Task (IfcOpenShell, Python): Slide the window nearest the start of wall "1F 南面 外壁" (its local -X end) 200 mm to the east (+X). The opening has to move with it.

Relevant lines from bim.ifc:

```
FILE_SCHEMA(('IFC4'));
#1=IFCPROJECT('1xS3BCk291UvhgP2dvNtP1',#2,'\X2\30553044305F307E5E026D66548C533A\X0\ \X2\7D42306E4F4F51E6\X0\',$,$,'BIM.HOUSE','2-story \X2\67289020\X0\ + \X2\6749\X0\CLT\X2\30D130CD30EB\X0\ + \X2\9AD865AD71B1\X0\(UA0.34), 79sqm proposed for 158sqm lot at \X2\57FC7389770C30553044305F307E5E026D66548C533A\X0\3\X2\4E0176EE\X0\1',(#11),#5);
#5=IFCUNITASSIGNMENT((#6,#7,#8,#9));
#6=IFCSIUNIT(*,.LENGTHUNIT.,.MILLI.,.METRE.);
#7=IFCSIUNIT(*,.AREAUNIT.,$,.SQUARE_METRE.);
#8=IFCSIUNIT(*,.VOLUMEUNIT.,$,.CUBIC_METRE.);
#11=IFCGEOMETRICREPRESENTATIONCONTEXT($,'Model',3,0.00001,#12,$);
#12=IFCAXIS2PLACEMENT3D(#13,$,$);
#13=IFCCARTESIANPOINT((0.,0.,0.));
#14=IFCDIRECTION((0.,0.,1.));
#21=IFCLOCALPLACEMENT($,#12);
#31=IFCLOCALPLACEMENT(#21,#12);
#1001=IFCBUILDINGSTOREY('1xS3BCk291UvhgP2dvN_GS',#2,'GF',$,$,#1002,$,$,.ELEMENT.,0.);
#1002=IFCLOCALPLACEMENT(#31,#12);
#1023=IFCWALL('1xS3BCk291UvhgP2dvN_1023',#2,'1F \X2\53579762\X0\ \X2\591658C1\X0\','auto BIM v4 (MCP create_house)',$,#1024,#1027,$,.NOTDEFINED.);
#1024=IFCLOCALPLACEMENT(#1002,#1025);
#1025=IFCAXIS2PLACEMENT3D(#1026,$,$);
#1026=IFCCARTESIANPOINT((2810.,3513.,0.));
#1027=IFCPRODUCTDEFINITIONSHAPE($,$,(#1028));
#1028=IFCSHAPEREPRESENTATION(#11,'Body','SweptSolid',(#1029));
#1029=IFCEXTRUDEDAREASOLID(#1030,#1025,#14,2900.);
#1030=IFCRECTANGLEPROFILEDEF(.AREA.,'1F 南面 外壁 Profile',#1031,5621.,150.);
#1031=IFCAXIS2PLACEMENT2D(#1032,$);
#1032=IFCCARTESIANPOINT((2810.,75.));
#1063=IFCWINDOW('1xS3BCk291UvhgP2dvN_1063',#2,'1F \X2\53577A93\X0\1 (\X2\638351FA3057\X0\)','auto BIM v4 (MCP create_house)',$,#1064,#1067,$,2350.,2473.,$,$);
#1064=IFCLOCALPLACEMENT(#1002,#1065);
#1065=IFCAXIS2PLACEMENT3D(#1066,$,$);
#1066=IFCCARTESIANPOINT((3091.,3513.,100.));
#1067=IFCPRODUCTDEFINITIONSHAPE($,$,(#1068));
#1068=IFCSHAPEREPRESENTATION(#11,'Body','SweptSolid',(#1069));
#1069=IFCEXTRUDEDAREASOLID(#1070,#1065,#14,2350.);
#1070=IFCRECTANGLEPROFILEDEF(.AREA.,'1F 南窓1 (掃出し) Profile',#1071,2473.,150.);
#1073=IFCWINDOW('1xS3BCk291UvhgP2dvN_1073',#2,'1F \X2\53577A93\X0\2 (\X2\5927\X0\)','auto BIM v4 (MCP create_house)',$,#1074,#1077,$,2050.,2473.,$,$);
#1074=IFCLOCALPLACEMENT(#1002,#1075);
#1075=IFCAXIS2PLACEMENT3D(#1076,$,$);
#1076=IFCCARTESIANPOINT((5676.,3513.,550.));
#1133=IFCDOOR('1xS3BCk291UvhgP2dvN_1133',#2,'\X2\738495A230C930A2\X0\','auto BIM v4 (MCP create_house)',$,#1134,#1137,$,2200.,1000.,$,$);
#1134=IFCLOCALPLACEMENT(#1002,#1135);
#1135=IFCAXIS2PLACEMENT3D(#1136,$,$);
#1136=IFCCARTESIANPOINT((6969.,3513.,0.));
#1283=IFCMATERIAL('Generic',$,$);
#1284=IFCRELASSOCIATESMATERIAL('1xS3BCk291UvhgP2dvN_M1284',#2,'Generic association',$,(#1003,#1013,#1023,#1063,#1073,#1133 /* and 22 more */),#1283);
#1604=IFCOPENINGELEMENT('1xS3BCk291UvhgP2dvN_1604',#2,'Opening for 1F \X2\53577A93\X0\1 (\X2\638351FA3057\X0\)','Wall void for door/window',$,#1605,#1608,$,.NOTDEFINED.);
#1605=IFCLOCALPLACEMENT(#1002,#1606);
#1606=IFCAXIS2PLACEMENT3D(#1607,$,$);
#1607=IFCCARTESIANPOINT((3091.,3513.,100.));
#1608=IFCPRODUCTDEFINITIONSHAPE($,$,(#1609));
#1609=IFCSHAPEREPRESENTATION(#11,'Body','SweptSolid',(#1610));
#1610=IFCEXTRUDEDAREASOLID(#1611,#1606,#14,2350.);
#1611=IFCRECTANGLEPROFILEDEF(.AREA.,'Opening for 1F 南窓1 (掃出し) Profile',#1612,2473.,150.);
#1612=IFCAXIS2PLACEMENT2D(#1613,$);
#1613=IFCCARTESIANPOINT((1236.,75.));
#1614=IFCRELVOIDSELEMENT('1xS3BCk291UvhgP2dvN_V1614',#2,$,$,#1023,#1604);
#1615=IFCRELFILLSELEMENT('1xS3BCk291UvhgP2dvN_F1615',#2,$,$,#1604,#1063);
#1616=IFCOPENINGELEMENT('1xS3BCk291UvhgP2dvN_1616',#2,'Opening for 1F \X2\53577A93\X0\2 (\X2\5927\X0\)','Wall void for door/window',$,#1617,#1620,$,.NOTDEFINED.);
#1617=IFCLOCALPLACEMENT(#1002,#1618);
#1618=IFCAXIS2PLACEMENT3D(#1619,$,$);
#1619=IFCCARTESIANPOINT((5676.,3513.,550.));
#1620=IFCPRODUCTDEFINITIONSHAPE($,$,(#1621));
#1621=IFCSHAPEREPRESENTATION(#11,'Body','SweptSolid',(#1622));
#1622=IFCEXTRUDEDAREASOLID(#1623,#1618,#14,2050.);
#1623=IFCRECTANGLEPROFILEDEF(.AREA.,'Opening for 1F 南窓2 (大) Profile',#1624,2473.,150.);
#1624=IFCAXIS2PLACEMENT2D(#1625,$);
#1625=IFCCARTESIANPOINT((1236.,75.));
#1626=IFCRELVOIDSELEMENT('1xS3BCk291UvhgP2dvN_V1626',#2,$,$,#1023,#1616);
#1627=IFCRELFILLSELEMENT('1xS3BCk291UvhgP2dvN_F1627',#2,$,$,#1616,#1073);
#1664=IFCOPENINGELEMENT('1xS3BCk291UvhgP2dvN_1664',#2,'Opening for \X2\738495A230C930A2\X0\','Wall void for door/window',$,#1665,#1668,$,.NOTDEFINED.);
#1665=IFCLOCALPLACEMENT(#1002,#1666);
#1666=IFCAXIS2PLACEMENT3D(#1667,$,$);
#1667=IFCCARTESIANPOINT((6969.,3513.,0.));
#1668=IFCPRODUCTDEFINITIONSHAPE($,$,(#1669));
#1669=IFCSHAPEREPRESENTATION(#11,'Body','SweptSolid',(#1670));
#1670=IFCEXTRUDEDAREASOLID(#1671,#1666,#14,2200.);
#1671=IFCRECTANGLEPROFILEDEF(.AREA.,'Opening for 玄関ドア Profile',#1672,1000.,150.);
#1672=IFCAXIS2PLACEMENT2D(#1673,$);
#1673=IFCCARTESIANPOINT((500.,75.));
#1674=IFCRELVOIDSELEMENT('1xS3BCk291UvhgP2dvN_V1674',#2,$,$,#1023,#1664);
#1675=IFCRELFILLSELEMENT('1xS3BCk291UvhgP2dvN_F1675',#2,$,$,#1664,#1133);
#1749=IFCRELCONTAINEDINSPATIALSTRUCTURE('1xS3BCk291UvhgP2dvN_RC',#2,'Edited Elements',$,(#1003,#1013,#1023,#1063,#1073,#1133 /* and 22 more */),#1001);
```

```python
import ifcopenshell
import ifcopenshell.api.geometry
import ifcopenshell.util.placement

model = ifcopenshell.open("bim.ifc")

window = model.by_guid("1xS3BCk291UvhgP2dvN_1063")
opening = window.FillsVoids[0].RelatingOpeningElement
wall = opening.VoidsElements[0].RelatingBuildingElement

wall_matrix = ifcopenshell.util.placement.get_local_placement(wall.ObjectPlacement)
shift = wall_matrix[:3, 0] * 200.0
before = ifcopenshell.util.placement.get_local_placement(window.ObjectPlacement)[:3, 3].copy()

# The window is not placed relative to its opening, so move both.
for product in (opening, window):
    matrix = ifcopenshell.util.placement.get_local_placement(product.ObjectPlacement)
    matrix[:3, 3] += shift
    ifcopenshell.api.geometry.edit_object_placement(model, product=product, matrix=matrix, is_si=False)

after = ifcopenshell.util.placement.get_local_placement(window.ObjectPlacement)[:3, 3]
print("window moved by", (after - before).round(3) + 0.0)

model.write("bim_edited.ifc")
```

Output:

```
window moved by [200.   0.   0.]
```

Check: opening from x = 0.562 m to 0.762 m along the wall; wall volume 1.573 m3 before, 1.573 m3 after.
